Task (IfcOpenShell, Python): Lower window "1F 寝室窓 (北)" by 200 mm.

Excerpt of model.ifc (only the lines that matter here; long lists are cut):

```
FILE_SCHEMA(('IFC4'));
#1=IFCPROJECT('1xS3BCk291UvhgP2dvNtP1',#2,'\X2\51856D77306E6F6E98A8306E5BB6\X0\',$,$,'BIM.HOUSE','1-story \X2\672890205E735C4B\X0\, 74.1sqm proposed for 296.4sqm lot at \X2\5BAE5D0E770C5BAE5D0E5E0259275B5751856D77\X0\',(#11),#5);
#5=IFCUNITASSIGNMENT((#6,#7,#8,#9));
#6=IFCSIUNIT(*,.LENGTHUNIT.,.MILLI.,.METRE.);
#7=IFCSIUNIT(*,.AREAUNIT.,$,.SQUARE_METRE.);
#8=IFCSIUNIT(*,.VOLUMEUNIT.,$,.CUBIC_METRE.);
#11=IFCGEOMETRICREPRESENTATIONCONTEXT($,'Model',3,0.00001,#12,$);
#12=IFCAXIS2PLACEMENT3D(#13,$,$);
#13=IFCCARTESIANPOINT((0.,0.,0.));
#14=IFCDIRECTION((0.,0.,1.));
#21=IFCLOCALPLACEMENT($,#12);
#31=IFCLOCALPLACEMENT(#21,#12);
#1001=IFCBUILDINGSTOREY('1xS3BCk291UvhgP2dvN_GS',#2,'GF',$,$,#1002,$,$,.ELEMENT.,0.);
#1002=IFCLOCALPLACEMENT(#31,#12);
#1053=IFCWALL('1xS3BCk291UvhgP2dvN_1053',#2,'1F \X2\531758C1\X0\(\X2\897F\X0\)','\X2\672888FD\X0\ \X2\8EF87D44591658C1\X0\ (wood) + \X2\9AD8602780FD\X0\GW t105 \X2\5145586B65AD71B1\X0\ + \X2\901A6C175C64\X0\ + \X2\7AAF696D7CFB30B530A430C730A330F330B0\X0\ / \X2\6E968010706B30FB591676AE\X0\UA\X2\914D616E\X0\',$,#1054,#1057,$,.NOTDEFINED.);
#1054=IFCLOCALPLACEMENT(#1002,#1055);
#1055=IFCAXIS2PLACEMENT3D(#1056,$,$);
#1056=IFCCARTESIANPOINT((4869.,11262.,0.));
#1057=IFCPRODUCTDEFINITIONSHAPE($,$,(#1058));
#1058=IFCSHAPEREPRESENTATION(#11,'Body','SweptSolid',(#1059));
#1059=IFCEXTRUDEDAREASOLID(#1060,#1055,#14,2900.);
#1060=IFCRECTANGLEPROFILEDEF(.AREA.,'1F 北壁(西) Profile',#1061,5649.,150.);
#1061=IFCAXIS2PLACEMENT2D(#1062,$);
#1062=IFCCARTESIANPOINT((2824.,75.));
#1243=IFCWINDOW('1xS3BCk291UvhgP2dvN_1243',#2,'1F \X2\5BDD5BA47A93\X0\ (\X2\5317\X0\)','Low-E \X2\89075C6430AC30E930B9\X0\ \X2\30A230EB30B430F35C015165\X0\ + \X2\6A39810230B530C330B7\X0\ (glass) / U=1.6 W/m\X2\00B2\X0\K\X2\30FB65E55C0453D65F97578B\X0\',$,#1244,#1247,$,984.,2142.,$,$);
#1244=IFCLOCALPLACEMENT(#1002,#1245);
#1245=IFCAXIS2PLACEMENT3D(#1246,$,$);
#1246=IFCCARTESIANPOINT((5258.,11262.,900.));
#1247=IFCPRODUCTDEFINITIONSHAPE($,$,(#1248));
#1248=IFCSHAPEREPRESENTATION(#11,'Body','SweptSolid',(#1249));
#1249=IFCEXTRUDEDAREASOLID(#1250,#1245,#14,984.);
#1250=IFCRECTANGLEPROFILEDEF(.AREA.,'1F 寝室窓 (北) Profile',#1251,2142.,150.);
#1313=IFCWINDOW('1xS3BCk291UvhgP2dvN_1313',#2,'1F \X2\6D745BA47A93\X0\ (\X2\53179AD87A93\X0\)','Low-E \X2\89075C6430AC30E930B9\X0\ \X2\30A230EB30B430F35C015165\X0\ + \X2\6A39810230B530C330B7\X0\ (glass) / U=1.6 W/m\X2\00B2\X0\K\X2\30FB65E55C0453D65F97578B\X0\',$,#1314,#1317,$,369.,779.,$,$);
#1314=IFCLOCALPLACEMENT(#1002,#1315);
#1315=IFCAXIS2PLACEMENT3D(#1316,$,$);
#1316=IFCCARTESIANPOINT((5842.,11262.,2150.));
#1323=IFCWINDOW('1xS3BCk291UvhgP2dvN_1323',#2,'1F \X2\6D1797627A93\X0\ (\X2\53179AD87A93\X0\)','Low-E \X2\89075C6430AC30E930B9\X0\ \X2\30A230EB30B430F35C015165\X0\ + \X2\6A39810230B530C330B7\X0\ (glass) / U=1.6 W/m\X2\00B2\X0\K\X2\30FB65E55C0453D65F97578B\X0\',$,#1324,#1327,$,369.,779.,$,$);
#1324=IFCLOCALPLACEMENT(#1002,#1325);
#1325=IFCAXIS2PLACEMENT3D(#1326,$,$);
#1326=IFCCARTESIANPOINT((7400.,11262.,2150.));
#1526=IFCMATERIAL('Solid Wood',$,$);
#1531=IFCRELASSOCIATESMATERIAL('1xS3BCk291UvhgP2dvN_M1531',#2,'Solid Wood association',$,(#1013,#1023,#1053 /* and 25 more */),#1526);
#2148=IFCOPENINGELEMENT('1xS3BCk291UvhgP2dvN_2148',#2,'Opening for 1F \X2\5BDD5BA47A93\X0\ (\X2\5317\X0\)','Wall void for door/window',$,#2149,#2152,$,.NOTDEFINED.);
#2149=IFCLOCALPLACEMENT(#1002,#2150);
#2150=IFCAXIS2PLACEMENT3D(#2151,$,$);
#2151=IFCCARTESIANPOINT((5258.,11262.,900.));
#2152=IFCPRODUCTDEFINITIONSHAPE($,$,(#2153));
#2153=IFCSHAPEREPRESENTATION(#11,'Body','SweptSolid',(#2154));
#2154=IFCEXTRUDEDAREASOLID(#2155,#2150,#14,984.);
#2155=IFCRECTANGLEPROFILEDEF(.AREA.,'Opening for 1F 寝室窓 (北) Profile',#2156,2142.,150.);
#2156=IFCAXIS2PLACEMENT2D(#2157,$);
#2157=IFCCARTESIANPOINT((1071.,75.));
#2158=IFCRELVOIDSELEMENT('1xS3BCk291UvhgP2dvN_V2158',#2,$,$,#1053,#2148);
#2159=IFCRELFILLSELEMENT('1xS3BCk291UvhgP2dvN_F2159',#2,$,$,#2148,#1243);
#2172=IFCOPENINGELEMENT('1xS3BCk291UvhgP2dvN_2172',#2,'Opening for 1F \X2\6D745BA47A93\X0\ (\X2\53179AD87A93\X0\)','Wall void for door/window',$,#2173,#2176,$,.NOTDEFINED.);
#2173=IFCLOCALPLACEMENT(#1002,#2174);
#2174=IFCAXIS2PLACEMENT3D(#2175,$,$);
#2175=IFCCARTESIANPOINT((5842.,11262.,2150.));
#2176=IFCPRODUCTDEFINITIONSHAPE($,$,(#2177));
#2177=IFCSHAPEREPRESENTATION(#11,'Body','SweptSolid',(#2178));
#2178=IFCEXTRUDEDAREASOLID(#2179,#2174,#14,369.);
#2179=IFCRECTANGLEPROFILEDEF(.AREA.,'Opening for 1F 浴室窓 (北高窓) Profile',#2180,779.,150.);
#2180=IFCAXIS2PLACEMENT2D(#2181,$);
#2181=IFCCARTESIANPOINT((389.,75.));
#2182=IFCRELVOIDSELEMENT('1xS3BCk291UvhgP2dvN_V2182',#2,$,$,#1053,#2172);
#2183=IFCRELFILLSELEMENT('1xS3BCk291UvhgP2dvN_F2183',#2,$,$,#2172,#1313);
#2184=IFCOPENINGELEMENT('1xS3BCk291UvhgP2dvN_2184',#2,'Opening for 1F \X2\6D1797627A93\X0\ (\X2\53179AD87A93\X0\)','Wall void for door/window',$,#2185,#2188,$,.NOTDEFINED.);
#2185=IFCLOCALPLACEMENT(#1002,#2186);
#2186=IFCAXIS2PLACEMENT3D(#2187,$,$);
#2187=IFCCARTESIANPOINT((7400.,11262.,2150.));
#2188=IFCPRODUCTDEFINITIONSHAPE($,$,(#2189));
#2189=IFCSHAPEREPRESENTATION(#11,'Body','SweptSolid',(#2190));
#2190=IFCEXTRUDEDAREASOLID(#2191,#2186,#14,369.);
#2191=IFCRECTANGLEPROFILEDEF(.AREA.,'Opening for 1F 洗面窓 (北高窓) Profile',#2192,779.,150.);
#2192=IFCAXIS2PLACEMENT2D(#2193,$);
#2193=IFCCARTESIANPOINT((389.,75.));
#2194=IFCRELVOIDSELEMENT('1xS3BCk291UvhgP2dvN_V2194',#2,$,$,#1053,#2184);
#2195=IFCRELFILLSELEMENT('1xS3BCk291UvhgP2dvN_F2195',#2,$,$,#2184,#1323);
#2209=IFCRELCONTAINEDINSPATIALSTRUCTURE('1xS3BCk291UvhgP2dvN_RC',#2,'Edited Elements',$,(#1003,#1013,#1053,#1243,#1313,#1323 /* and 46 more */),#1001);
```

```python
import numpy as np
import ifcopenshell
import ifcopenshell.api.geometry
import ifcopenshell.util.placement
import ifcopenshell.util.unit

model = ifcopenshell.open("model.ifc")
unit_scale = ifcopenshell.util.unit.calculate_unit_scale(model)

window = model.by_id(1243)
opening = window.FillsVoids[0].RelatingOpeningElement
dz = -0.2 / unit_scale

shift = np.array([0.0, 0.0, dz])
# The window is not placed relative to its opening, so move both.
for product in (opening, window):
    matrix = ifcopenshell.util.placement.get_local_placement(product.ObjectPlacement)
    matrix[:3, 3] += shift
    ifcopenshell.api.geometry.edit_object_placement(model, product=product, matrix=matrix, is_si=False)

print(f"moved by {dz * unit_scale:+.3f} m")

model.write("model_rev.ifc")
```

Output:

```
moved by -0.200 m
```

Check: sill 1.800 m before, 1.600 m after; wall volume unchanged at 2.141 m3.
